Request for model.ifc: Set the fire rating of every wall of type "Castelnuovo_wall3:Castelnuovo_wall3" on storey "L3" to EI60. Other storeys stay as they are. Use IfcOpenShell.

First a look at what the model holds.

```python
import ifcopenshell
import ifcopenshell.util.element

model = ifcopenshell.open("model.ifc")
print(model.schema)
storey = next(s for s in model.by_type("IfcBuildingStorey") if s.Name == "L3")
walls = [e for e in ifcopenshell.util.element.get_decomposition(storey) if e.is_a("IfcWall")]
seen = {}
for e in walls:
    element_type = ifcopenshell.util.element.get_type(e)
    key = (element_type.Name if element_type != e and element_type else None, ifcopenshell.util.element.get_pset(e, "Pset_WallCommon", "FireRating"))
    seen[key] = seen.get(key, 0) + 1
for (name, value), count in sorted(seen.items(), key=str):
    print(count, "x", name, "|", value)
```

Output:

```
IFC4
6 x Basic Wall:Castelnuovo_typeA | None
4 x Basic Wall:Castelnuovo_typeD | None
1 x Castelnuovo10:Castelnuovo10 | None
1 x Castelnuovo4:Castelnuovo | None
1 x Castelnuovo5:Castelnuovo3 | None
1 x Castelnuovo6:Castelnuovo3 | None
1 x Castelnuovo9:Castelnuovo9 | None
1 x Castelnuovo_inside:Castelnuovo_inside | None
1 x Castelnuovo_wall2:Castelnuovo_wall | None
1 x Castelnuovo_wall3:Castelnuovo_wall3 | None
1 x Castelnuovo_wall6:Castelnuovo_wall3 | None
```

```python
import ifcopenshell
import ifcopenshell.api.pset
import ifcopenshell.util.element

model = ifcopenshell.open("model.ifc")

storey = next(s for s in model.by_type("IfcBuildingStorey") if s.Name == "L3")
walls = [e for e in ifcopenshell.util.element.get_decomposition(storey) if e.is_a("IfcWall")]

count = 0
for e in walls:
    element_type = ifcopenshell.util.element.get_type(e)
    if element_type in (None, e) or element_type.Name != "Castelnuovo_wall3:Castelnuovo_wall3":
        continue
    # add_pset returns the element's existing set when there is one.
    pset = ifcopenshell.api.pset.add_pset(model, product=e, name="Pset_WallCommon")
    ifcopenshell.api.pset.edit_pset(model, pset=pset, properties={"FireRating": "EI60"})
    count += 1

print(count, "walls updated")

model.write("model_edited.ifc")
```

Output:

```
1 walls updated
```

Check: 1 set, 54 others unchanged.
